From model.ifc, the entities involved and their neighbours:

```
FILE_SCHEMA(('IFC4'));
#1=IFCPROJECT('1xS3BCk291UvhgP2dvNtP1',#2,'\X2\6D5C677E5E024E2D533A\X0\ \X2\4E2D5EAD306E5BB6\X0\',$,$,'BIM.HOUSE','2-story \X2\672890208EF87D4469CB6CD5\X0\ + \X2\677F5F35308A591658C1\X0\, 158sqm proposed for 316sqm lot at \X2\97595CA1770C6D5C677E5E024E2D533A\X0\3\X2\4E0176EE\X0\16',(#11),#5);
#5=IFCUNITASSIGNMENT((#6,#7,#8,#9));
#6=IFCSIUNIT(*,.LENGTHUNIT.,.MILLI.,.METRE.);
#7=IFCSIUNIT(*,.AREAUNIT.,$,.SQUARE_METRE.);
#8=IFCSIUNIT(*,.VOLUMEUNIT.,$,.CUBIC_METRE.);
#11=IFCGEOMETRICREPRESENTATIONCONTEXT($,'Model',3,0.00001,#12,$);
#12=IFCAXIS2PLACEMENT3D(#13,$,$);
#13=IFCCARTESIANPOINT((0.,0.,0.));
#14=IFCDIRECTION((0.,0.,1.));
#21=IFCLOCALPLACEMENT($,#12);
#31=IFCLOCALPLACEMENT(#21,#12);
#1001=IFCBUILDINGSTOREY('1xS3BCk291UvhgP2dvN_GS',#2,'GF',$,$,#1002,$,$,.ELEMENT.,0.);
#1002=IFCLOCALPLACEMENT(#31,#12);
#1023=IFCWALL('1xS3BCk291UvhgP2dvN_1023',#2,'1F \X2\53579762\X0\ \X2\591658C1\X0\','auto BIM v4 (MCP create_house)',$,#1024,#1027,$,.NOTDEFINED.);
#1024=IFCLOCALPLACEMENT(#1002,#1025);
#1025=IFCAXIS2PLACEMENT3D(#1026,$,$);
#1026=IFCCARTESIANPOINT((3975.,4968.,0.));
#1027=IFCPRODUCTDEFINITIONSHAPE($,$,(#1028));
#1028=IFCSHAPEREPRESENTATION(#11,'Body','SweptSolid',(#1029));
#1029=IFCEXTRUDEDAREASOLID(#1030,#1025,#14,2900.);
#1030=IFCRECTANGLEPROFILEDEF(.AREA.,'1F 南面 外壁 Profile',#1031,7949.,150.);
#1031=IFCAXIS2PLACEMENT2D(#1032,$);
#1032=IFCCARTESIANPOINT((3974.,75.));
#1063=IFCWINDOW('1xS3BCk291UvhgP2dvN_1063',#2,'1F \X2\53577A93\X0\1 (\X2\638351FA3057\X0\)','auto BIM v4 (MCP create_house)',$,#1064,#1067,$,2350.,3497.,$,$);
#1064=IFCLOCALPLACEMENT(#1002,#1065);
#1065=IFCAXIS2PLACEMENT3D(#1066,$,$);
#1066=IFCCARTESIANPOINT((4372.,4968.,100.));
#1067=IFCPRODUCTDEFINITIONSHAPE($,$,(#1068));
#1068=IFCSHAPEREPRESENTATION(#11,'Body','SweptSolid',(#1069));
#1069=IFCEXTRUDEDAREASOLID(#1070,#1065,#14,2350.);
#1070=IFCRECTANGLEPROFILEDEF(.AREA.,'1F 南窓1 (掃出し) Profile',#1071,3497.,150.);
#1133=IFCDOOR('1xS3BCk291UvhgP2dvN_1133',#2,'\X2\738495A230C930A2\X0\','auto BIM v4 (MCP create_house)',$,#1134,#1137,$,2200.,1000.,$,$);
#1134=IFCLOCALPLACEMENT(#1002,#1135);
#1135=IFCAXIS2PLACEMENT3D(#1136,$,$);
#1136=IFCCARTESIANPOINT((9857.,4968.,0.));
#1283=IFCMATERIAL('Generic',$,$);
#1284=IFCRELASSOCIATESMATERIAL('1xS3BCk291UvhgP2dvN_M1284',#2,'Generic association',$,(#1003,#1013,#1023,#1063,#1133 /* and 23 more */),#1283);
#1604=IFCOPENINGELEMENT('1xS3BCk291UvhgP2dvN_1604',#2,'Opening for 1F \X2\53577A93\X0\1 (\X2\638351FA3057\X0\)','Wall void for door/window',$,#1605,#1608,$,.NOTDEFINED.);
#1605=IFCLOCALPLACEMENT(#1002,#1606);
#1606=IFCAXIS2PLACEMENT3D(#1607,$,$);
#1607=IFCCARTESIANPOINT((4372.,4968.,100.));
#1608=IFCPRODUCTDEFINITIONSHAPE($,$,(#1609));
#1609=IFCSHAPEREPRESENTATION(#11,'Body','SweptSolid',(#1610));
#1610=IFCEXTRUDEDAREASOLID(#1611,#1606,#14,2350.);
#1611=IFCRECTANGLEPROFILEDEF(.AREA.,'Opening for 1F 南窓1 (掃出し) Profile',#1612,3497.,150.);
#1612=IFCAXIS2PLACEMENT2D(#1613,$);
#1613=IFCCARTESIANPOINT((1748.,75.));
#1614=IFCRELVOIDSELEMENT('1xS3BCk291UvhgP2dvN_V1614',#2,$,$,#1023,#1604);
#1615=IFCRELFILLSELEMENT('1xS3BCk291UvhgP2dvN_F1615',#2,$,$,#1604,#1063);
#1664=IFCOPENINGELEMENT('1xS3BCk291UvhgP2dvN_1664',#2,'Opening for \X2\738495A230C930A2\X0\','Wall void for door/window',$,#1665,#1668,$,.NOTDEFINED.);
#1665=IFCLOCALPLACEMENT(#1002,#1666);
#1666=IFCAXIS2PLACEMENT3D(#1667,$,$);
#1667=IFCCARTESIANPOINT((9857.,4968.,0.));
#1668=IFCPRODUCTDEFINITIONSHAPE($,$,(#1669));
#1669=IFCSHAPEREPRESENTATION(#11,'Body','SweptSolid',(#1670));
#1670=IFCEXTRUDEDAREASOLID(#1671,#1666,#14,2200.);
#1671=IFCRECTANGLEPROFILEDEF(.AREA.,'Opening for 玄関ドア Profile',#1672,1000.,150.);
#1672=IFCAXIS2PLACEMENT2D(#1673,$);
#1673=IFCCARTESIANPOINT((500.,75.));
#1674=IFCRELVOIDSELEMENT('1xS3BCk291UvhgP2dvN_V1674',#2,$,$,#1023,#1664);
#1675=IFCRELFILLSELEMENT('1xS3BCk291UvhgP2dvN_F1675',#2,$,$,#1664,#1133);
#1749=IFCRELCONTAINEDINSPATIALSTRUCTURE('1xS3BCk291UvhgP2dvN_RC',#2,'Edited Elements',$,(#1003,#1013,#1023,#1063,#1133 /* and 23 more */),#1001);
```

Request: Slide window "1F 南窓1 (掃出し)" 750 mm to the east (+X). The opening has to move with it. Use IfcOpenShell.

```python
import ifcopenshell
import ifcopenshell.api.geometry
import ifcopenshell.util.placement
import ifcopenshell.util.unit

model = ifcopenshell.open("model.ifc")
unit_scale = ifcopenshell.util.unit.calculate_unit_scale(model)

window = model.by_id(1063)
opening = window.FillsVoids[0].RelatingOpeningElement
wall = opening.VoidsElements[0].RelatingBuildingElement

wall_matrix = ifcopenshell.util.placement.get_local_placement(wall.ObjectPlacement)
shift = wall_matrix[:3, 0] * 0.75 / unit_scale
before = ifcopenshell.util.placement.get_local_placement(window.ObjectPlacement)[:3, 3].copy()

# The window is not placed relative to its opening, so move both.
for product in (opening, window):
    matrix = ifcopenshell.util.placement.get_local_placement(product.ObjectPlacement)
    matrix[:3, 3] += shift
    ifcopenshell.api.geometry.edit_object_placement(model, product=product, matrix=matrix, is_si=False)

after = ifcopenshell.util.placement.get_local_placement(window.ObjectPlacement)[:3, 3]
print("window moved by", (after - before).round(3) + 0.0)

model.write("model_rev.ifc")
```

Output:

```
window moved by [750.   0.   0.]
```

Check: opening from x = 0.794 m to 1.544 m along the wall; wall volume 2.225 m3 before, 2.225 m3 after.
